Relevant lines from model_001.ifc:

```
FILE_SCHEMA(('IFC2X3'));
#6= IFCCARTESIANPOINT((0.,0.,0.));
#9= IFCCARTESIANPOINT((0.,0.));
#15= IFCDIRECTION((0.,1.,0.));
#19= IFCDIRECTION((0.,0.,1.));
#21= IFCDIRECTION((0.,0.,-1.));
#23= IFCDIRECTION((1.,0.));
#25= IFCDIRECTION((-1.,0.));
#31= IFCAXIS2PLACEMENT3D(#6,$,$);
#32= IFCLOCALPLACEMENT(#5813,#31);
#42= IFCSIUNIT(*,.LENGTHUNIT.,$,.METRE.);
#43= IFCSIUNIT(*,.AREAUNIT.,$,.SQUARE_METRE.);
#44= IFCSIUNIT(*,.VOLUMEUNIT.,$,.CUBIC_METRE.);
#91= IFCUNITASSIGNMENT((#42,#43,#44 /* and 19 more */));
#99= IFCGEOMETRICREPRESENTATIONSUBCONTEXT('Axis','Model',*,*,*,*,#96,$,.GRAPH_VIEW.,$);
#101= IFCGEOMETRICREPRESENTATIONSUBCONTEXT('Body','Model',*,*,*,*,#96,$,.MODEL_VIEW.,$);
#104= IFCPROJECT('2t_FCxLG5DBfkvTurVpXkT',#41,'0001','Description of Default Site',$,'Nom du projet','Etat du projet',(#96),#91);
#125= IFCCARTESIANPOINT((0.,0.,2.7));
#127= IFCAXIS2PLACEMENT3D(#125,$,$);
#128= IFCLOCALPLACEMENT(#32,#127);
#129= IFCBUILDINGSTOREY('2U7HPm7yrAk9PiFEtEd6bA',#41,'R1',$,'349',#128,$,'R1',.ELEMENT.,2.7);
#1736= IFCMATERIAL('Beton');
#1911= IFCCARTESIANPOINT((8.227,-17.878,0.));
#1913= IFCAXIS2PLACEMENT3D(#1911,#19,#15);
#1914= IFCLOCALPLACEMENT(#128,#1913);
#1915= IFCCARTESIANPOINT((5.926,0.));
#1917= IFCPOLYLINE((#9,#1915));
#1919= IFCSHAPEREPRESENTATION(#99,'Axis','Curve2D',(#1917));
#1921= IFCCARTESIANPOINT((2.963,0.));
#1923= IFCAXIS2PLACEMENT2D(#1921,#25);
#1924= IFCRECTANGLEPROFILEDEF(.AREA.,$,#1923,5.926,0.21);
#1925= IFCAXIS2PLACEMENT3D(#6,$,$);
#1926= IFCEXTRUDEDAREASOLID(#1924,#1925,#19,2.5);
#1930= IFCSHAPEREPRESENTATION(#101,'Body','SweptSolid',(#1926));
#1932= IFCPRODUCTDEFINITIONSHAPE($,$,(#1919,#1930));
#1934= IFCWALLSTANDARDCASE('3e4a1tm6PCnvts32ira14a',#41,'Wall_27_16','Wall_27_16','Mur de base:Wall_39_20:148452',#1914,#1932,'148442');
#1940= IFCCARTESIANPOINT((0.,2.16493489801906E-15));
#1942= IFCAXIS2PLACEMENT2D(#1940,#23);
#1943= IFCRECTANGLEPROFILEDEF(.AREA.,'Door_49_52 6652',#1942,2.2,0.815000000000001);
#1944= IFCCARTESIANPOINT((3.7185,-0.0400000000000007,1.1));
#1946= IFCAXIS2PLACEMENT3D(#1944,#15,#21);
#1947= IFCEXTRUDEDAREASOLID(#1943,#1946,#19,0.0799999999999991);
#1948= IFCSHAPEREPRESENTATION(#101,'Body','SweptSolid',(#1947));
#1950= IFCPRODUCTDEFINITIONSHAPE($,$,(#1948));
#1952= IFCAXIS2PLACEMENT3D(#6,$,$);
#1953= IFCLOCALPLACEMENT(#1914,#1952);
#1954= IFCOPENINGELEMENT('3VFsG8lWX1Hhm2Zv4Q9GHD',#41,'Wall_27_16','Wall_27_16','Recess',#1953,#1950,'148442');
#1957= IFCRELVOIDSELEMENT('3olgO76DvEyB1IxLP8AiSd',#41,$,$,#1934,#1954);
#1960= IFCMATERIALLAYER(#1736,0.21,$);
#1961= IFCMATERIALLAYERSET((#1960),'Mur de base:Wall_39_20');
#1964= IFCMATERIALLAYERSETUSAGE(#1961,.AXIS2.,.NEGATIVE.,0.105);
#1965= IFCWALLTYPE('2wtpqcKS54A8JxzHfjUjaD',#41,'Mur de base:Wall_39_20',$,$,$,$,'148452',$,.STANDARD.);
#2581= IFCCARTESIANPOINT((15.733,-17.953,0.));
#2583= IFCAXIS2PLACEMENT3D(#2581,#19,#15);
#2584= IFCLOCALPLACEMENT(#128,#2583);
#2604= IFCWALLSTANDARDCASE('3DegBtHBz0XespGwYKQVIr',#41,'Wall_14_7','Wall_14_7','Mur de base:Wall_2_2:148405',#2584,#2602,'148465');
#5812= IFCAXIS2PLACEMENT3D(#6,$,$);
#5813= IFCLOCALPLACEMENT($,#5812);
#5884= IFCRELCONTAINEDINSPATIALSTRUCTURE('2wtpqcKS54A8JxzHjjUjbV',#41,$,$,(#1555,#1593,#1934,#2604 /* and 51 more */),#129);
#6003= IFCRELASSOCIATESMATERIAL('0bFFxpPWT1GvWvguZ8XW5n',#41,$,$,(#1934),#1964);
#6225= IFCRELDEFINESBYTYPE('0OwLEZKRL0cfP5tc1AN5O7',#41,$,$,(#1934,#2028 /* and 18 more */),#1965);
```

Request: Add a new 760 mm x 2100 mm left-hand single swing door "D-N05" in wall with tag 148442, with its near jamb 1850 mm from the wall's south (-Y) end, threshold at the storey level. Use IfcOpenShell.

```python
import numpy as np
import ifcopenshell
import ifcopenshell.api.feature
import ifcopenshell.api.geometry
import ifcopenshell.api.root
import ifcopenshell.api.spatial
import ifcopenshell.api.type
import ifcopenshell.geom
import ifcopenshell.util.element
import ifcopenshell.util.placement
import ifcopenshell.util.representation
import ifcopenshell.util.shape
import ifcopenshell.util.unit

model = ifcopenshell.open("model_001.ifc")
unit_scale = ifcopenshell.util.unit.calculate_unit_scale(model)
settings = ifcopenshell.geom.settings()


def volume(element):
    """Net volume in cubic metres, openings subtracted."""
    shape = ifcopenshell.geom.create_shape(settings, element)
    return ifcopenshell.util.shape.get_volume(shape.geometry)


wall = model.by_guid("3e4a1tm6PCnvts32ira14a")
storey = ifcopenshell.util.element.get_container(wall, ifc_class="IfcBuildingStorey")
context = ifcopenshell.util.representation.get_context(model, "Model", "Body", "MODEL_VIEW")
before = volume(wall)

width, height, from_end, sill = 0.76, 2.1, 1.85, 0.0  # metres

# The wall runs along its own X axis, and the end named is its -X end.
wall_shape = ifcopenshell.geom.create_shape(settings, wall)
x, y, z = ifcopenshell.util.shape.get_vertices(wall_shape.geometry).T
start = x.min() + from_end
face, thickness = float(y.min()), float(y.max() - y.min())
wall_matrix = ifcopenshell.util.placement.get_local_placement(wall.ObjectPlacement)
level = ifcopenshell.util.placement.get_local_placement(storey.ObjectPlacement)[2, 3]


def in_wall(x, y):
    """Placement at x, y metres in the wall's axes, at sill height."""
    matrix = wall_matrix.copy()
    matrix[:, 3] = wall_matrix @ np.array([x / unit_scale, y / unit_scale, 0.0, 1.0])
    matrix[2, 3] = level + sill / unit_scale
    return matrix


# Opening: a box that overshoots both wall faces by 50 mm.
opening = ifcopenshell.api.root.create_entity(model, ifc_class="IfcOpeningElement")
box = ifcopenshell.api.geometry.add_wall_representation(
    model, context=context, length=width, height=height, thickness=thickness + 0.1
)
ifcopenshell.api.geometry.assign_representation(model, product=opening, representation=box)
ifcopenshell.api.geometry.edit_object_placement(model, product=opening, matrix=in_wall(start, face - 0.05), is_si=False)
ifcopenshell.api.feature.add_feature(model, feature=opening, element=wall)

door = ifcopenshell.api.root.create_entity(model, ifc_class="IfcDoor", name="D-N05")
door.OverallWidth, door.OverallHeight = width / unit_scale, height / unit_scale
body = ifcopenshell.api.geometry.add_door_representation(
    model,
    context=context,
    overall_width=door.OverallWidth,
    overall_height=door.OverallHeight,
    operation_type="SINGLE_SWING_LEFT",
    lining_properties={"LiningDepth": thickness / unit_scale, "ThresholdDepth": thickness / unit_scale},
)
ifcopenshell.api.geometry.assign_representation(model, product=door, representation=body)
ifcopenshell.api.spatial.assign_container(model, products=[door], relating_structure=storey)
fills = ifcopenshell.api.feature.add_filling(model, opening=opening, element=door)
fills.OwnerHistory = door.OwnerHistory  # required in IFC2X3

# IFC2X3 keeps the operation on the door style.
style = ifcopenshell.api.root.create_entity(model, ifc_class="IfcDoorStyle", name="D-N05")
style.OperationType, style.ConstructionType = "SINGLE_SWING_LEFT", "NOTDEFINED"
style.ParameterTakesPrecedence = style.Sizeable = False
ifcopenshell.api.type.assign_type(model, related_objects=[door], relating_type=style)

# The lining spans the wall, so the door starts at the wall face.
ifcopenshell.api.geometry.edit_object_placement(model, product=door, matrix=in_wall(start, face), is_si=False)

after = volume(wall)

print(f"wall volume {before:.3f} -> {after:.3f} m3")

model.write("model_001_edited.ifc")
```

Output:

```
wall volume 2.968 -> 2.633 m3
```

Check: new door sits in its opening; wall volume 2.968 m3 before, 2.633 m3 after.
